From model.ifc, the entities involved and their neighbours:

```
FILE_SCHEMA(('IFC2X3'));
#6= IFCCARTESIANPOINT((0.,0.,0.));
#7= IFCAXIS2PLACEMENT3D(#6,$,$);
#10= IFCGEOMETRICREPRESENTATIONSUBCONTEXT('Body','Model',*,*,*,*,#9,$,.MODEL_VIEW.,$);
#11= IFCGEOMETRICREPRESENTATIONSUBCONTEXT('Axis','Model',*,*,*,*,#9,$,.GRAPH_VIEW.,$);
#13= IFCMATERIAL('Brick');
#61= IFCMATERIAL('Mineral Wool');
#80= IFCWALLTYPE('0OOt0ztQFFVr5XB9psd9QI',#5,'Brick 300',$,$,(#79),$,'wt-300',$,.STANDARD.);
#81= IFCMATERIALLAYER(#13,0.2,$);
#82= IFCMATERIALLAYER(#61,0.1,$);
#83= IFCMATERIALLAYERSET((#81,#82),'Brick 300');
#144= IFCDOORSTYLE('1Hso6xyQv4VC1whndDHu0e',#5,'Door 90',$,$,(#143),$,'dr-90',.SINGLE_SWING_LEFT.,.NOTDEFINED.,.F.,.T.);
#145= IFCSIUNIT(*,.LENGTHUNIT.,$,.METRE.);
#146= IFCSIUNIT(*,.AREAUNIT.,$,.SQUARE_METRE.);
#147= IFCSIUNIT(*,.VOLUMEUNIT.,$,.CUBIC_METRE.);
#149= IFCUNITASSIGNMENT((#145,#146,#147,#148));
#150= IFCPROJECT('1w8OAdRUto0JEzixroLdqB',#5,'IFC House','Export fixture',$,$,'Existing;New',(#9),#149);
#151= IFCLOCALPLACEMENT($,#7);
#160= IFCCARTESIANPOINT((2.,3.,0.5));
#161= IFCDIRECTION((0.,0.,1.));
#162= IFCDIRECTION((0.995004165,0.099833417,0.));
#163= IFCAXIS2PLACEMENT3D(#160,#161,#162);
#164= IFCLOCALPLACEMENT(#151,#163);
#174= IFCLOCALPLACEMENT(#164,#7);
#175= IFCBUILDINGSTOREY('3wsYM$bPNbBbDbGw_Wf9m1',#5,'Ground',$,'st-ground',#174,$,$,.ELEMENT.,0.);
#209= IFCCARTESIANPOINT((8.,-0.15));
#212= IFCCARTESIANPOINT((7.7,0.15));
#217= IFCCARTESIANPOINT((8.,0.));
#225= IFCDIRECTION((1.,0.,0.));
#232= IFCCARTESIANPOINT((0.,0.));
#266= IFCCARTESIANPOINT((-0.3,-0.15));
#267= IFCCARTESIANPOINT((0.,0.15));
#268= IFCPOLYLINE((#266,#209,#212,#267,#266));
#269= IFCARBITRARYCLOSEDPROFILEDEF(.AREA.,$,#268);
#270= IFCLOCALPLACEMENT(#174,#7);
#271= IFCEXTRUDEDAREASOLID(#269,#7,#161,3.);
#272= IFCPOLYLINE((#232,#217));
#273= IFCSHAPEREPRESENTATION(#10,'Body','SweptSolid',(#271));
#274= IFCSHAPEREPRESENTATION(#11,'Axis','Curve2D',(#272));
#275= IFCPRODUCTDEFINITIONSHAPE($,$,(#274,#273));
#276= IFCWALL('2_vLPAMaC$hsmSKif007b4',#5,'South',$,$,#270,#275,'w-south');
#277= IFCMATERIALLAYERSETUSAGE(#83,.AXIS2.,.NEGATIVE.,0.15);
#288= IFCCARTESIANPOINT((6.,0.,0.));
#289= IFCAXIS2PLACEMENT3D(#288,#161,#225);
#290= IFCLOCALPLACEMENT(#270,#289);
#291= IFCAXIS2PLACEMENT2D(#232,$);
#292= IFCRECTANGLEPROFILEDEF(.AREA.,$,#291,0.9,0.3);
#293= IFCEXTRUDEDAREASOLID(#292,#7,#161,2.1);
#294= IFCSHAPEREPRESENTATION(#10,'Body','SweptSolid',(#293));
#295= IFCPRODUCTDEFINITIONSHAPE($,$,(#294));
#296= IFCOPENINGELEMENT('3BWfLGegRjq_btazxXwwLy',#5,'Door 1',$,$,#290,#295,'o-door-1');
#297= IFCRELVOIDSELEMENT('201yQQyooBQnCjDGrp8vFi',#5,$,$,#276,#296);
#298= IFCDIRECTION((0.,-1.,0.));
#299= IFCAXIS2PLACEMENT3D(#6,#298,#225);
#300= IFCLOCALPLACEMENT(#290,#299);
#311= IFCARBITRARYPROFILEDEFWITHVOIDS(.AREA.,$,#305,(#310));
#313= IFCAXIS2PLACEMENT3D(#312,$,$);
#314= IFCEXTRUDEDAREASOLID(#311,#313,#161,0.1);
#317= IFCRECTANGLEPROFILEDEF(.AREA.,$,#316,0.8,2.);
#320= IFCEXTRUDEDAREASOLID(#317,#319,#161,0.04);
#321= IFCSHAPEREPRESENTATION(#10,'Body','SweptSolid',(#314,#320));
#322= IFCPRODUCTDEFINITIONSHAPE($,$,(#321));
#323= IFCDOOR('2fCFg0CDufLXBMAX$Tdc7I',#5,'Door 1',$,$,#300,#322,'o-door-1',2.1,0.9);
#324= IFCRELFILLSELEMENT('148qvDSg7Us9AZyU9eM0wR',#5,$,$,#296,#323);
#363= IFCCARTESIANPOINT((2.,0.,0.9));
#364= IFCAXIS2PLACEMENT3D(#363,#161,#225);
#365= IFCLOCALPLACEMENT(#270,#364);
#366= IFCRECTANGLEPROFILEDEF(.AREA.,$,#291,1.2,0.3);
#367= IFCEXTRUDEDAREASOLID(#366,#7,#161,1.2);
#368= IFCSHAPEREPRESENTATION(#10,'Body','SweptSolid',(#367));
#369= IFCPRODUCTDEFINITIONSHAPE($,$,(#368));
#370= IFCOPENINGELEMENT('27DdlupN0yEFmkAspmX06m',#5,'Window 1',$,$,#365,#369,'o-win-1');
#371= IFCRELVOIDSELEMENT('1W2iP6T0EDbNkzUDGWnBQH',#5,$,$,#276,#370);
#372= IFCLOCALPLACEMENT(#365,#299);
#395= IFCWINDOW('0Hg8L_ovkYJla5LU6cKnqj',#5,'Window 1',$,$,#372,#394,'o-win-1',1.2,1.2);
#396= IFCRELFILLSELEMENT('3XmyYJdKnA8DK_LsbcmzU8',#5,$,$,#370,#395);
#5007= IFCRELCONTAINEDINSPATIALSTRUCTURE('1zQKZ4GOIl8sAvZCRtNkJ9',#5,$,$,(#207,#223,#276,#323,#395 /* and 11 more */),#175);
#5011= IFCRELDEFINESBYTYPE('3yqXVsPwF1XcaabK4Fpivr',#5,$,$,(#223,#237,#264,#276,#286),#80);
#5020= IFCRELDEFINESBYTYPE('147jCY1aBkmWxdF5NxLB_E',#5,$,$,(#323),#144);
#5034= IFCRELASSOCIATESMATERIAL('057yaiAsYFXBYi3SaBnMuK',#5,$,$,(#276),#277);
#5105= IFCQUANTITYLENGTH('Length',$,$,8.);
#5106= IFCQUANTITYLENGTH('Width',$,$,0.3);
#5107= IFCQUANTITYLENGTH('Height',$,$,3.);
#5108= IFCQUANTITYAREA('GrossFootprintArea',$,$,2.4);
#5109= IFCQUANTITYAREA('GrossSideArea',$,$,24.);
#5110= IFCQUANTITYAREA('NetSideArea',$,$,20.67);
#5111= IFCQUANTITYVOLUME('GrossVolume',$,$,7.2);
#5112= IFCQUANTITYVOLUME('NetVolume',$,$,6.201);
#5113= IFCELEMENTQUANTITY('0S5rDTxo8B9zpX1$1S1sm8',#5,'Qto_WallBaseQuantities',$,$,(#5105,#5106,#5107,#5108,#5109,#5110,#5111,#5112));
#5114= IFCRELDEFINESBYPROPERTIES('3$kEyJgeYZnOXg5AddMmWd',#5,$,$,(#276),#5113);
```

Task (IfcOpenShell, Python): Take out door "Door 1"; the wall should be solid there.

```python
import ifcopenshell
import ifcopenshell.api.feature
import ifcopenshell.api.pset
import ifcopenshell.api.root
import ifcopenshell.geom
import ifcopenshell.util.element
import ifcopenshell.util.shape
import ifcopenshell.util.unit

model = ifcopenshell.open("model.ifc")
area_scale = ifcopenshell.util.unit.calculate_unit_scale(model, "AREAUNIT")
volume_scale = ifcopenshell.util.unit.calculate_unit_scale(model, "VOLUMEUNIT")
settings = ifcopenshell.geom.settings()


def volume(element):
    """Net volume in cubic metres, openings subtracted."""
    shape = ifcopenshell.geom.create_shape(settings, element)
    return ifcopenshell.util.shape.get_volume(shape.geometry)


door = model.by_id(323)
opening = door.FillsVoids[0].RelatingOpeningElement
wall = opening.VoidsElements[0].RelatingBuildingElement
before = volume(wall)

ifcopenshell.api.root.remove_product(model, product=door)
ifcopenshell.api.feature.remove_feature(model, feature=opening)

after = volume(wall)
thickness = 0.3  # wall thickness in metres

# Update the wall's stored quantities.
qto = model.by_id(ifcopenshell.util.element.get_pset(wall, "Qto_WallBaseQuantities", should_inherit=False)["id"])
ifcopenshell.api.pset.edit_qto(model, qto=qto, properties={
    "NetSideArea": after / thickness / area_scale,
    "NetVolume": after / volume_scale,
})

print(f"wall volume {before:.3f} -> {after:.3f} m3")

model.write("model_edited.ifc")
```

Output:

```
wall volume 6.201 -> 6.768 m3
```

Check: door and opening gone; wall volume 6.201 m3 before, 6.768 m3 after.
